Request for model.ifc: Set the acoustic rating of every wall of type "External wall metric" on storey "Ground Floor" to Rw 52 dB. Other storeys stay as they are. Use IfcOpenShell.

First a look at what the model holds.

```python
import ifcopenshell
import ifcopenshell.util.element

model = ifcopenshell.open("model.ifc")
print(model.schema)
storey = next(s for s in model.by_type("IfcBuildingStorey") if s.Name == "Ground Floor")
walls = [e for e in ifcopenshell.util.element.get_decomposition(storey) if e.is_a("IfcWall")]
seen = {}
for e in walls:
    element_type = ifcopenshell.util.element.get_type(e)
    key = (element_type.Name if element_type != e and element_type else None, ifcopenshell.util.element.get_pset(e, "Pset_WallCommon", "AcousticRating"))
    seen[key] = seen.get(key, 0) + 1
for (name, value), count in sorted(seen.items(), key=str):
    print(count, "x", name, "|", value)
```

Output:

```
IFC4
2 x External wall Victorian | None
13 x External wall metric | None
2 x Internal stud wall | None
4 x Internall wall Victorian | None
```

```python
import ifcopenshell
import ifcopenshell.api.pset
import ifcopenshell.util.element

model = ifcopenshell.open("model.ifc")

storey = next(s for s in model.by_type("IfcBuildingStorey") if s.Name == "Ground Floor")
walls = [e for e in ifcopenshell.util.element.get_decomposition(storey) if e.is_a("IfcWall")]

count = 0
for e in walls:
    element_type = ifcopenshell.util.element.get_type(e)
    if element_type in (None, e) or element_type.Name != "External wall metric":
        continue
    # add_pset returns the element's existing set when there is one.
    pset = ifcopenshell.api.pset.add_pset(model, product=e, name="Pset_WallCommon")
    ifcopenshell.api.pset.edit_pset(model, pset=pset, properties={"AcousticRating": "Rw 52 dB"})
    count += 1

print(count, "walls updated")

model.write("model_v2.ifc")
```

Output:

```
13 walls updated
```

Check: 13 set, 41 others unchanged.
